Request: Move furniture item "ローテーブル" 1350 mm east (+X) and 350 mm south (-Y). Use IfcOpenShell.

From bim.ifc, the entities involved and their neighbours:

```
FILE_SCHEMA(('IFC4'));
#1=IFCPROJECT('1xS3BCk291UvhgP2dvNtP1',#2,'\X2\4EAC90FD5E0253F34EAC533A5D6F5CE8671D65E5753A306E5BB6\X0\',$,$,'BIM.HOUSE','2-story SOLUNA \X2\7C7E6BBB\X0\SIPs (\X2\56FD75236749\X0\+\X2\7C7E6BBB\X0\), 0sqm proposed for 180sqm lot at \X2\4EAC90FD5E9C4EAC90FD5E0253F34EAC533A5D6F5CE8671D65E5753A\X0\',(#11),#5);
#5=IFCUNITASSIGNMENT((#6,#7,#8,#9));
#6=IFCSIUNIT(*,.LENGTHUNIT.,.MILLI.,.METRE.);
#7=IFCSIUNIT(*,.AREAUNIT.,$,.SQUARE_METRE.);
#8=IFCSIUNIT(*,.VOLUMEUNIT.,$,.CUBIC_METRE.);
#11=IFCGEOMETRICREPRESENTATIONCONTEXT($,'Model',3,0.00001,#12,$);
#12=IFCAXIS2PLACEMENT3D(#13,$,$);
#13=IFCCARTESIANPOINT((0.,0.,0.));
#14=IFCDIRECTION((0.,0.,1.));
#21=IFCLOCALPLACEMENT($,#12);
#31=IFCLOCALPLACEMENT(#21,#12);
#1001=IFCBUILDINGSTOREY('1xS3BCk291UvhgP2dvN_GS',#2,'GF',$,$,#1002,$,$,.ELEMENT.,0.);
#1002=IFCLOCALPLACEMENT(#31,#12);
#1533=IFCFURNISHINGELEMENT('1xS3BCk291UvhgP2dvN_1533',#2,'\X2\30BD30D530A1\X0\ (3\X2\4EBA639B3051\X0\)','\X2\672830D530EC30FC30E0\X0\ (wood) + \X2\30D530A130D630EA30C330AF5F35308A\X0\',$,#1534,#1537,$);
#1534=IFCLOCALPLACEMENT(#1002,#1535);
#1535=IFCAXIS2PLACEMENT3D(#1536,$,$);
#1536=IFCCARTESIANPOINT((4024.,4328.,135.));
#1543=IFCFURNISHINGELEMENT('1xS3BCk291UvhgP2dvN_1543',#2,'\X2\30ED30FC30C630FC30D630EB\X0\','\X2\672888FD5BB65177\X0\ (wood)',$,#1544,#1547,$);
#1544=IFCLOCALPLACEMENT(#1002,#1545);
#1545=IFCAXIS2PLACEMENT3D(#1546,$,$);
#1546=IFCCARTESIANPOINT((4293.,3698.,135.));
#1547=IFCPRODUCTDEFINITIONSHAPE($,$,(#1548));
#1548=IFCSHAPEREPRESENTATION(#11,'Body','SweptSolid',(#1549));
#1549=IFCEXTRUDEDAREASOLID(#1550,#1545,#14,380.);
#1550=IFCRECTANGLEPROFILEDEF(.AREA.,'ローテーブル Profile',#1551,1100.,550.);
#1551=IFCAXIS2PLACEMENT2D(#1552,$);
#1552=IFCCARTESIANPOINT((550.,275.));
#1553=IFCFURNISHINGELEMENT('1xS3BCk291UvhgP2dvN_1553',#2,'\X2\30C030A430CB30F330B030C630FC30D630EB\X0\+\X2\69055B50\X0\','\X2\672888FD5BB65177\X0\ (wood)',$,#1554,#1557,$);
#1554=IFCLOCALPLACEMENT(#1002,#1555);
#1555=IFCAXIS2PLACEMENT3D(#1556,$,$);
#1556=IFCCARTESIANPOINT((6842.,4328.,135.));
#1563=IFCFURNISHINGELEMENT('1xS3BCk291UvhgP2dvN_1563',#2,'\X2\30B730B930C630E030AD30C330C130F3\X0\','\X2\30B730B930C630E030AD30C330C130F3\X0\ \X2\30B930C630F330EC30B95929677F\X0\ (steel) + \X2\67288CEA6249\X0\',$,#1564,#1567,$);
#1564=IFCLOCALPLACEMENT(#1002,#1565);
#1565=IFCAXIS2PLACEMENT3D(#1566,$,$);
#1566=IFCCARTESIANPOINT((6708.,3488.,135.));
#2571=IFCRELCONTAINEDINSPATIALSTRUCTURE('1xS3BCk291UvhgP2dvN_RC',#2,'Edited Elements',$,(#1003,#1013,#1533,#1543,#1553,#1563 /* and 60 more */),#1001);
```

```python
import ifcopenshell
import ifcopenshell.api.geometry
import ifcopenshell.util.placement
import ifcopenshell.util.unit

model = ifcopenshell.open("bim.ifc")
unit_scale = ifcopenshell.util.unit.calculate_unit_scale(model)

item = model.by_guid("1xS3BCk291UvhgP2dvN_1543")
matrix = ifcopenshell.util.placement.get_local_placement(item.ObjectPlacement)
matrix[0, 3] += 1.35 / unit_scale
matrix[1, 3] -= 0.35 / unit_scale
ifcopenshell.api.geometry.edit_object_placement(model, product=item, matrix=matrix, is_si=False)

print(ifcopenshell.util.placement.get_local_placement(item.ObjectPlacement).round(3) + 0.0)

model.write("bim-out.ifc")
```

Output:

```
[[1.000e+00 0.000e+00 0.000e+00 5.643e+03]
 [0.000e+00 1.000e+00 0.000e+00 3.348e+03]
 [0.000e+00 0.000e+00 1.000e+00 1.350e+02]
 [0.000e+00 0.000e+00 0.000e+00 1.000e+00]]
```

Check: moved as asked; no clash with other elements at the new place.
